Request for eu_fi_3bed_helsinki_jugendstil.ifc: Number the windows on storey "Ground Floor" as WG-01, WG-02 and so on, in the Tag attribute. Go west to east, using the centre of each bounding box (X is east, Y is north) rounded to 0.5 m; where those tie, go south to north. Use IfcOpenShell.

First a look at what the model holds.

```python
import ifcopenshell
import ifcopenshell.util.element
import ifcopenshell.util.placement

model = ifcopenshell.open("eu_fi_3bed_helsinki_jugendstil.ifc")
print(model.schema)
storey = next(s for s in model.by_type("IfcBuildingStorey") if s.Name == "Ground Floor")
windows = [e for e in ifcopenshell.util.element.get_decomposition(storey) if e.is_a("IfcWindow")]
for e in sorted(windows, key=lambda e: e.id()):
    origin = ifcopenshell.util.placement.get_local_placement(e.ObjectPlacement)[:3, 3]
    print(e.id(), e.Tag, e.Name, origin.round(2) + 0.0, sep=" | ")
```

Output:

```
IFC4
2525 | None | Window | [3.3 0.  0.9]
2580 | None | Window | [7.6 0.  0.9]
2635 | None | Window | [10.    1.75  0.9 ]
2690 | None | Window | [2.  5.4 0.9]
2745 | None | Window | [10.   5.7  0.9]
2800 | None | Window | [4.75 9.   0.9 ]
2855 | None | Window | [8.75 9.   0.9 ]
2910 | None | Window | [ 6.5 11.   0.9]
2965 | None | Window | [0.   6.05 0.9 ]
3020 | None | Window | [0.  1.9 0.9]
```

```python
import ifcopenshell
import ifcopenshell.geom
import ifcopenshell.util.element
import ifcopenshell.util.shape

model = ifcopenshell.open("eu_fi_3bed_helsinki_jugendstil.ifc")
settings = ifcopenshell.geom.settings()
settings.set("use-world-coords", True)


def centre(element):
    shape = ifcopenshell.geom.create_shape(settings, element)
    return ifcopenshell.util.shape.get_bbox_centroid(shape.geometry)


storey = next(s for s in model.by_type("IfcBuildingStorey") if s.Name == "Ground Floor")
windows = [e for e in ifcopenshell.util.element.get_decomposition(storey) if e.is_a("IfcWindow")]

# Insertion points can sit at a corner or the storey origin, so sort by the geometry (in metres).
centres = {e: centre(e) for e in windows}
windows.sort(key=lambda e: (round(centres[e][0] / 0.5), centres[e][1]))

for i, e in enumerate(windows, start=1):
    number = f"WG-{i:02d}"
    e.Tag = number
    print(e.id(), number)

model.write("eu_fi_3bed_helsinki_jugendstil_rev.ifc")
```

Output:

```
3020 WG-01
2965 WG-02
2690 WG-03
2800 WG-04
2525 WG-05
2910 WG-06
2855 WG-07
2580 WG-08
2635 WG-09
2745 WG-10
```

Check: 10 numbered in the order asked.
